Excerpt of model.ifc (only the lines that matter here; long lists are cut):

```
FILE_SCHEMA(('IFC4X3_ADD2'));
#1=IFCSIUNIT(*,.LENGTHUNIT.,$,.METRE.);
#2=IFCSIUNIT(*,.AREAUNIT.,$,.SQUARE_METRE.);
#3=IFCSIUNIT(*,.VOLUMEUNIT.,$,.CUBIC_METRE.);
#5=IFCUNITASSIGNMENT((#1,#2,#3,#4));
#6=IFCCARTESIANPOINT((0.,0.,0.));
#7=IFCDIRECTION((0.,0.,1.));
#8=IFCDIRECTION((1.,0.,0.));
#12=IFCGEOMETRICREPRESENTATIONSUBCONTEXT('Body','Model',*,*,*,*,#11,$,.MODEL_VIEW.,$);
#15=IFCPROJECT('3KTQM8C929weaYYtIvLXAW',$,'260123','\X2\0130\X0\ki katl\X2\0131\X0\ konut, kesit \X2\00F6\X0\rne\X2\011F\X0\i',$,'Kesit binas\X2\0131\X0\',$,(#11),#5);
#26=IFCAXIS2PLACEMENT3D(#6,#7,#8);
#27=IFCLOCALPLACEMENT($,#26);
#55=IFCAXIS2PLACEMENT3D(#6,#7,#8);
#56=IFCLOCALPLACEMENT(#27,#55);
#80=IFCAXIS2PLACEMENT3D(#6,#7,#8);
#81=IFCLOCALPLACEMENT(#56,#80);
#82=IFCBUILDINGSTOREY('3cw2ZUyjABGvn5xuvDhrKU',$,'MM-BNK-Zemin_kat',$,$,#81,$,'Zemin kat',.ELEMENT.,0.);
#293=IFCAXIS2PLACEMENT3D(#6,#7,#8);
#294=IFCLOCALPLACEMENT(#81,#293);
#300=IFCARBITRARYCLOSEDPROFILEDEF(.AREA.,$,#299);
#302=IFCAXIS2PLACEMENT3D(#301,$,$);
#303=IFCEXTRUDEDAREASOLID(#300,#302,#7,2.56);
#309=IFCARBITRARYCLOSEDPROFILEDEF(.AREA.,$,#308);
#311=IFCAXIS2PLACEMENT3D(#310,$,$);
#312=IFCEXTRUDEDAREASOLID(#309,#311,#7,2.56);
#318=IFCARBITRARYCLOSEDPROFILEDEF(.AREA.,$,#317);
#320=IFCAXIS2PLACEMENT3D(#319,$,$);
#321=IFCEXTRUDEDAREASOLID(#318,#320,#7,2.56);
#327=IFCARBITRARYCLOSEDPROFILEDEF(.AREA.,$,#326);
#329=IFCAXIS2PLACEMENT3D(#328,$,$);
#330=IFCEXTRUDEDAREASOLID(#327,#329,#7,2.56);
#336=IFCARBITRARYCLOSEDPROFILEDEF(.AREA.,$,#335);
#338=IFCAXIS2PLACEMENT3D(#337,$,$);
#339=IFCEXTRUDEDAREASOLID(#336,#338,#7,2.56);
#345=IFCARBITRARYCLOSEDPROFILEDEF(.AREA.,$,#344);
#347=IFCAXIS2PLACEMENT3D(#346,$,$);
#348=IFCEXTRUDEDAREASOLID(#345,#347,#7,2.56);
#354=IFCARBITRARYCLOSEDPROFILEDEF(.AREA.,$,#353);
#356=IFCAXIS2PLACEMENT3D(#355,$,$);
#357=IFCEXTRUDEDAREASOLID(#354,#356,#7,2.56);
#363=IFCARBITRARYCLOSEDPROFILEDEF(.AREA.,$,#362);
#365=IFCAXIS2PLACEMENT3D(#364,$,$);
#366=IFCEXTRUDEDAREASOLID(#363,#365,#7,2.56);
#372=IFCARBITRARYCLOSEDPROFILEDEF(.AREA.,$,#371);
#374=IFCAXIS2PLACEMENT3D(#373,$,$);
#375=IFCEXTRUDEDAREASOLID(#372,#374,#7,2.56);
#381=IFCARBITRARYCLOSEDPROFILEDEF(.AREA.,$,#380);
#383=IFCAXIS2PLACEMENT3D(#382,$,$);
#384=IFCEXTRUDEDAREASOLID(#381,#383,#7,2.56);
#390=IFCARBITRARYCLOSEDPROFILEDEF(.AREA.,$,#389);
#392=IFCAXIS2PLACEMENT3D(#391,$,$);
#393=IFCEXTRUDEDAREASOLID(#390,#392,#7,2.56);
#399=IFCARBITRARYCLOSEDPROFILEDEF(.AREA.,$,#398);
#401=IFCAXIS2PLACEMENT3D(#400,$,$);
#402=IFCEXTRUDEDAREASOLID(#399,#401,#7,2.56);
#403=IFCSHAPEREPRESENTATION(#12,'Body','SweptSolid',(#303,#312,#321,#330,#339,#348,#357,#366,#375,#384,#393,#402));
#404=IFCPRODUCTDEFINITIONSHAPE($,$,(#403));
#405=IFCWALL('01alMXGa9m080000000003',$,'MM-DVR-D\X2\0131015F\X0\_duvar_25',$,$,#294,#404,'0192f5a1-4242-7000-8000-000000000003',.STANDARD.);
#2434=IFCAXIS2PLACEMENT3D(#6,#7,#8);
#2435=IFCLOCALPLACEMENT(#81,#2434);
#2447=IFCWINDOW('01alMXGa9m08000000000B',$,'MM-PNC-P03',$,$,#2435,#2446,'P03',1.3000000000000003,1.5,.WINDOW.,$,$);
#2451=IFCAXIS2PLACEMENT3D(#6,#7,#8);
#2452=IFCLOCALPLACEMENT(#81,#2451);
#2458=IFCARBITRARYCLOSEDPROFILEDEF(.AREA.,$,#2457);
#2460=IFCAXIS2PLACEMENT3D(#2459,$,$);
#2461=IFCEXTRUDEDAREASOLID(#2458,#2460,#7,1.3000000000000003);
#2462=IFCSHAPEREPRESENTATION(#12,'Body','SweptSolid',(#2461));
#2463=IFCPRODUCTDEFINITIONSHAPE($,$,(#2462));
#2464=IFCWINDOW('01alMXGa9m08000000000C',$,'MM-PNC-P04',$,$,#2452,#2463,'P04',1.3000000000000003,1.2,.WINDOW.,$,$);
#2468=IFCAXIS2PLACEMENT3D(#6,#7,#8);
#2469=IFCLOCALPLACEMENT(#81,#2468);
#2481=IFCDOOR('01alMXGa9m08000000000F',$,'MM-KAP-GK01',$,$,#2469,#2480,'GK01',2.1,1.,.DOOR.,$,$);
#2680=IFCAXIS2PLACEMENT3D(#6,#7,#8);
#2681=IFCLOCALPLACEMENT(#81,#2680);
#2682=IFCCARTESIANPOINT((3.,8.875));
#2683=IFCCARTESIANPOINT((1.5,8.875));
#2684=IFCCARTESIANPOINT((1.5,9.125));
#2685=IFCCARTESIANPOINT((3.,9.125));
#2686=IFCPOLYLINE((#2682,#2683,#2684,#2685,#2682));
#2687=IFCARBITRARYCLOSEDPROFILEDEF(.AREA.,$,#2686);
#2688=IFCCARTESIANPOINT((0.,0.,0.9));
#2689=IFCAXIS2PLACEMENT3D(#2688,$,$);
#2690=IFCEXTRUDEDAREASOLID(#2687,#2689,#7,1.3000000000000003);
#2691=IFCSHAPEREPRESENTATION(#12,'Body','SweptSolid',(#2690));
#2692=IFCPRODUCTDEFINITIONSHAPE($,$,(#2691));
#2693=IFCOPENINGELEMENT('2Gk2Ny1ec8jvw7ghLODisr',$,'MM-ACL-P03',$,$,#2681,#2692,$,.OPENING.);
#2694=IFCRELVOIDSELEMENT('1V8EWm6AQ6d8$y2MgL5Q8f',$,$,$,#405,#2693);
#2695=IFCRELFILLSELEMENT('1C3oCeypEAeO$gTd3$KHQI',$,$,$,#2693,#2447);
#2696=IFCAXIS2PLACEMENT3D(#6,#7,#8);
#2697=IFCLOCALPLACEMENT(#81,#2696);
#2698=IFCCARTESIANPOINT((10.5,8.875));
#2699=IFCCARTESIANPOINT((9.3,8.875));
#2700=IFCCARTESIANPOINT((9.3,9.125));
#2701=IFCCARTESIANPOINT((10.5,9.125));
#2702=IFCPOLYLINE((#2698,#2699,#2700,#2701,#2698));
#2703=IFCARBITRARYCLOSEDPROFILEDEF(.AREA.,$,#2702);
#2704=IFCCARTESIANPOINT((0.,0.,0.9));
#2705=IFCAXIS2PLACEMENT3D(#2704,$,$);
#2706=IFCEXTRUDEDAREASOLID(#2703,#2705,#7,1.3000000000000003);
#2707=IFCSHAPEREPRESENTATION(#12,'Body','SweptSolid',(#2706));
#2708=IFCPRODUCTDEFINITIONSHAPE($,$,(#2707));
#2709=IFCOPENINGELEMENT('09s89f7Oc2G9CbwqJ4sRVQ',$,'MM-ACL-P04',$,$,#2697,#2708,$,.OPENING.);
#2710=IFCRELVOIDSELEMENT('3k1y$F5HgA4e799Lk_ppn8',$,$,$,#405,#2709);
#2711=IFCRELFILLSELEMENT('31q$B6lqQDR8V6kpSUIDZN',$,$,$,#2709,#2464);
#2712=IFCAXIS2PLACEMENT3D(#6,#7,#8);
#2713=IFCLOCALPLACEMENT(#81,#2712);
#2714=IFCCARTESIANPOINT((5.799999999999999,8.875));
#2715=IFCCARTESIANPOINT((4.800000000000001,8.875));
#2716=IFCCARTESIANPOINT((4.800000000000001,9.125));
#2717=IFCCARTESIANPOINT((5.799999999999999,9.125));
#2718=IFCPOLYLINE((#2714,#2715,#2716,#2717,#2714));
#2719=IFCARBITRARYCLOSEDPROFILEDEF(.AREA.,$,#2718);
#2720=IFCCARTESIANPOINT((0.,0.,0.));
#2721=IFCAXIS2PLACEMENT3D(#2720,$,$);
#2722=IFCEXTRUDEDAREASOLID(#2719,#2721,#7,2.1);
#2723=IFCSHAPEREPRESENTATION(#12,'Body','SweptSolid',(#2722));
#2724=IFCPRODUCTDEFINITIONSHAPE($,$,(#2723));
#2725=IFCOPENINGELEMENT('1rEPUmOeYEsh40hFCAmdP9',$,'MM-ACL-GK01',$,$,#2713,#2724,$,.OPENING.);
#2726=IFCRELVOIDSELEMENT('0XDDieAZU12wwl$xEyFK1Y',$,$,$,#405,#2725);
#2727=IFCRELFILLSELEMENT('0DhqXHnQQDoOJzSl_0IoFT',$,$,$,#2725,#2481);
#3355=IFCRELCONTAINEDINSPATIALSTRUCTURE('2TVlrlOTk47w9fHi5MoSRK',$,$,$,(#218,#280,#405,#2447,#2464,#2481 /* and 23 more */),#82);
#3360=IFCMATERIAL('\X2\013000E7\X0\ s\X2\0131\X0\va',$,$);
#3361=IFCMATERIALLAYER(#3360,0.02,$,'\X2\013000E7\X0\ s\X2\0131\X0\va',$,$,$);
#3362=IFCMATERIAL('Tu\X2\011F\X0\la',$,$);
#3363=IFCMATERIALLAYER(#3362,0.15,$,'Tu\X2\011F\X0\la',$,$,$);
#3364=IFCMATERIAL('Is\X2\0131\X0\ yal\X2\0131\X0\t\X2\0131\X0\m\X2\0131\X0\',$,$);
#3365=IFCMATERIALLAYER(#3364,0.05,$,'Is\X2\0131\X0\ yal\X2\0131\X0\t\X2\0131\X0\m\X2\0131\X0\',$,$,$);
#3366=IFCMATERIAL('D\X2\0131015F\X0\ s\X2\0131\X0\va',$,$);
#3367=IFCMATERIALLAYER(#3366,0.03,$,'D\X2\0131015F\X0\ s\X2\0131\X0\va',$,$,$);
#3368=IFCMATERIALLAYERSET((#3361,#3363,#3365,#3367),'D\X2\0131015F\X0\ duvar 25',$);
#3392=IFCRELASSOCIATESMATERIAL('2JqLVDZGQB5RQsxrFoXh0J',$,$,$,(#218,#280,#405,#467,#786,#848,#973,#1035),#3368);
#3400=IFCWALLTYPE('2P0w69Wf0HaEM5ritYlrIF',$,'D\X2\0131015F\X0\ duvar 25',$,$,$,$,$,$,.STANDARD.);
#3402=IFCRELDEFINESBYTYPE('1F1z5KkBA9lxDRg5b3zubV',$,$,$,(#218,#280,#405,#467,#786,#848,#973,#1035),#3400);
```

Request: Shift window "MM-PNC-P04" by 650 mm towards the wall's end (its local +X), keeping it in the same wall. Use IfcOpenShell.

```python
import ifcopenshell
import ifcopenshell.api.geometry
import ifcopenshell.util.placement
import ifcopenshell.util.unit

model = ifcopenshell.open("model.ifc")
unit_scale = ifcopenshell.util.unit.calculate_unit_scale(model)

window = model.by_guid("01alMXGa9m08000000000C")
opening = window.FillsVoids[0].RelatingOpeningElement
wall = opening.VoidsElements[0].RelatingBuildingElement

wall_matrix = ifcopenshell.util.placement.get_local_placement(wall.ObjectPlacement)
shift = wall_matrix[:3, 0] * 0.65 / unit_scale
before = ifcopenshell.util.placement.get_local_placement(window.ObjectPlacement)[:3, 3].copy()

# The window is not placed relative to its opening, so move both.
for product in (opening, window):
    matrix = ifcopenshell.util.placement.get_local_placement(product.ObjectPlacement)
    matrix[:3, 3] += shift
    ifcopenshell.api.geometry.edit_object_placement(model, product=product, matrix=matrix, is_si=False)

after = ifcopenshell.util.placement.get_local_placement(window.ObjectPlacement)[:3, 3]
print("window moved by", (after - before).round(3) + 0.0)

model.write("model_edited.ifc")
```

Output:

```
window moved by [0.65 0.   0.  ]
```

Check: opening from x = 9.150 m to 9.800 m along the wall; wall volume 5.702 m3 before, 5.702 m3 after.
